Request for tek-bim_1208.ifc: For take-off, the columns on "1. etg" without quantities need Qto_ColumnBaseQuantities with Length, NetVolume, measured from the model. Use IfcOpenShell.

First a look at what the model holds.

```python
import ifcopenshell
import ifcopenshell.util.element
import ifcopenshell.util.unit

model = ifcopenshell.open("tek-bim_1208.ifc")
print(model.schema)
for unit_type in ("LENGTHUNIT", "AREAUNIT", "VOLUMEUNIT"):
    print(unit_type, ifcopenshell.util.unit.calculate_unit_scale(model, unit_type))
storey = next(s for s in model.by_type("IfcBuildingStorey") if s.Name == "1. etg")
columns = [e for e in ifcopenshell.util.element.get_decomposition(storey) if e.is_a("IfcColumn")]
for e in sorted(columns, key=lambda e: e.id()):
    print(e.id(), e.is_a(), e.Name, list(ifcopenshell.util.element.get_psets(e, qtos_only=True)), sep=" | ")
```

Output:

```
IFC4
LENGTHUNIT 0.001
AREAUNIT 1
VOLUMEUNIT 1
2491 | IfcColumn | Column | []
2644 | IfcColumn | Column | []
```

```python
import ifcopenshell
import ifcopenshell.api.pset
import ifcopenshell.geom
import ifcopenshell.util.element
import ifcopenshell.util.shape
import ifcopenshell.util.unit

model = ifcopenshell.open("tek-bim_1208.ifc")
unit_scale = ifcopenshell.util.unit.calculate_unit_scale(model)
volume_scale = ifcopenshell.util.unit.calculate_unit_scale(model, "VOLUMEUNIT")
settings = ifcopenshell.geom.settings()

storey = next(s for s in model.by_type("IfcBuildingStorey") if s.Name == "1. etg")
columns = [e for e in ifcopenshell.util.element.get_decomposition(storey) if e.is_a("IfcColumn")]

for e in sorted(columns, key=lambda e: e.id()):
    if ifcopenshell.util.element.get_psets(e, qtos_only=True, should_inherit=False):
        continue
    # Geometry comes back in metres, in the element's own axes.
    shape = ifcopenshell.geom.create_shape(settings, e)
    values = {
        "Length": ifcopenshell.util.shape.get_z(shape.geometry) / unit_scale,
        "NetVolume": ifcopenshell.util.shape.get_volume(shape.geometry) / volume_scale,
    }
    qto = ifcopenshell.api.pset.add_qto(model, product=e, name="Qto_ColumnBaseQuantities")
    ifcopenshell.api.pset.edit_qto(model, qto=qto, properties=values)
    print(e.id(), {k: round(v, 3) for k, v in values.items()})

model.write("tek-bim_1208_edited.ifc")
```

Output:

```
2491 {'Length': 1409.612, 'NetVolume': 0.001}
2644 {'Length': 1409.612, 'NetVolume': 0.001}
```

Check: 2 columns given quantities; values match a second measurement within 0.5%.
